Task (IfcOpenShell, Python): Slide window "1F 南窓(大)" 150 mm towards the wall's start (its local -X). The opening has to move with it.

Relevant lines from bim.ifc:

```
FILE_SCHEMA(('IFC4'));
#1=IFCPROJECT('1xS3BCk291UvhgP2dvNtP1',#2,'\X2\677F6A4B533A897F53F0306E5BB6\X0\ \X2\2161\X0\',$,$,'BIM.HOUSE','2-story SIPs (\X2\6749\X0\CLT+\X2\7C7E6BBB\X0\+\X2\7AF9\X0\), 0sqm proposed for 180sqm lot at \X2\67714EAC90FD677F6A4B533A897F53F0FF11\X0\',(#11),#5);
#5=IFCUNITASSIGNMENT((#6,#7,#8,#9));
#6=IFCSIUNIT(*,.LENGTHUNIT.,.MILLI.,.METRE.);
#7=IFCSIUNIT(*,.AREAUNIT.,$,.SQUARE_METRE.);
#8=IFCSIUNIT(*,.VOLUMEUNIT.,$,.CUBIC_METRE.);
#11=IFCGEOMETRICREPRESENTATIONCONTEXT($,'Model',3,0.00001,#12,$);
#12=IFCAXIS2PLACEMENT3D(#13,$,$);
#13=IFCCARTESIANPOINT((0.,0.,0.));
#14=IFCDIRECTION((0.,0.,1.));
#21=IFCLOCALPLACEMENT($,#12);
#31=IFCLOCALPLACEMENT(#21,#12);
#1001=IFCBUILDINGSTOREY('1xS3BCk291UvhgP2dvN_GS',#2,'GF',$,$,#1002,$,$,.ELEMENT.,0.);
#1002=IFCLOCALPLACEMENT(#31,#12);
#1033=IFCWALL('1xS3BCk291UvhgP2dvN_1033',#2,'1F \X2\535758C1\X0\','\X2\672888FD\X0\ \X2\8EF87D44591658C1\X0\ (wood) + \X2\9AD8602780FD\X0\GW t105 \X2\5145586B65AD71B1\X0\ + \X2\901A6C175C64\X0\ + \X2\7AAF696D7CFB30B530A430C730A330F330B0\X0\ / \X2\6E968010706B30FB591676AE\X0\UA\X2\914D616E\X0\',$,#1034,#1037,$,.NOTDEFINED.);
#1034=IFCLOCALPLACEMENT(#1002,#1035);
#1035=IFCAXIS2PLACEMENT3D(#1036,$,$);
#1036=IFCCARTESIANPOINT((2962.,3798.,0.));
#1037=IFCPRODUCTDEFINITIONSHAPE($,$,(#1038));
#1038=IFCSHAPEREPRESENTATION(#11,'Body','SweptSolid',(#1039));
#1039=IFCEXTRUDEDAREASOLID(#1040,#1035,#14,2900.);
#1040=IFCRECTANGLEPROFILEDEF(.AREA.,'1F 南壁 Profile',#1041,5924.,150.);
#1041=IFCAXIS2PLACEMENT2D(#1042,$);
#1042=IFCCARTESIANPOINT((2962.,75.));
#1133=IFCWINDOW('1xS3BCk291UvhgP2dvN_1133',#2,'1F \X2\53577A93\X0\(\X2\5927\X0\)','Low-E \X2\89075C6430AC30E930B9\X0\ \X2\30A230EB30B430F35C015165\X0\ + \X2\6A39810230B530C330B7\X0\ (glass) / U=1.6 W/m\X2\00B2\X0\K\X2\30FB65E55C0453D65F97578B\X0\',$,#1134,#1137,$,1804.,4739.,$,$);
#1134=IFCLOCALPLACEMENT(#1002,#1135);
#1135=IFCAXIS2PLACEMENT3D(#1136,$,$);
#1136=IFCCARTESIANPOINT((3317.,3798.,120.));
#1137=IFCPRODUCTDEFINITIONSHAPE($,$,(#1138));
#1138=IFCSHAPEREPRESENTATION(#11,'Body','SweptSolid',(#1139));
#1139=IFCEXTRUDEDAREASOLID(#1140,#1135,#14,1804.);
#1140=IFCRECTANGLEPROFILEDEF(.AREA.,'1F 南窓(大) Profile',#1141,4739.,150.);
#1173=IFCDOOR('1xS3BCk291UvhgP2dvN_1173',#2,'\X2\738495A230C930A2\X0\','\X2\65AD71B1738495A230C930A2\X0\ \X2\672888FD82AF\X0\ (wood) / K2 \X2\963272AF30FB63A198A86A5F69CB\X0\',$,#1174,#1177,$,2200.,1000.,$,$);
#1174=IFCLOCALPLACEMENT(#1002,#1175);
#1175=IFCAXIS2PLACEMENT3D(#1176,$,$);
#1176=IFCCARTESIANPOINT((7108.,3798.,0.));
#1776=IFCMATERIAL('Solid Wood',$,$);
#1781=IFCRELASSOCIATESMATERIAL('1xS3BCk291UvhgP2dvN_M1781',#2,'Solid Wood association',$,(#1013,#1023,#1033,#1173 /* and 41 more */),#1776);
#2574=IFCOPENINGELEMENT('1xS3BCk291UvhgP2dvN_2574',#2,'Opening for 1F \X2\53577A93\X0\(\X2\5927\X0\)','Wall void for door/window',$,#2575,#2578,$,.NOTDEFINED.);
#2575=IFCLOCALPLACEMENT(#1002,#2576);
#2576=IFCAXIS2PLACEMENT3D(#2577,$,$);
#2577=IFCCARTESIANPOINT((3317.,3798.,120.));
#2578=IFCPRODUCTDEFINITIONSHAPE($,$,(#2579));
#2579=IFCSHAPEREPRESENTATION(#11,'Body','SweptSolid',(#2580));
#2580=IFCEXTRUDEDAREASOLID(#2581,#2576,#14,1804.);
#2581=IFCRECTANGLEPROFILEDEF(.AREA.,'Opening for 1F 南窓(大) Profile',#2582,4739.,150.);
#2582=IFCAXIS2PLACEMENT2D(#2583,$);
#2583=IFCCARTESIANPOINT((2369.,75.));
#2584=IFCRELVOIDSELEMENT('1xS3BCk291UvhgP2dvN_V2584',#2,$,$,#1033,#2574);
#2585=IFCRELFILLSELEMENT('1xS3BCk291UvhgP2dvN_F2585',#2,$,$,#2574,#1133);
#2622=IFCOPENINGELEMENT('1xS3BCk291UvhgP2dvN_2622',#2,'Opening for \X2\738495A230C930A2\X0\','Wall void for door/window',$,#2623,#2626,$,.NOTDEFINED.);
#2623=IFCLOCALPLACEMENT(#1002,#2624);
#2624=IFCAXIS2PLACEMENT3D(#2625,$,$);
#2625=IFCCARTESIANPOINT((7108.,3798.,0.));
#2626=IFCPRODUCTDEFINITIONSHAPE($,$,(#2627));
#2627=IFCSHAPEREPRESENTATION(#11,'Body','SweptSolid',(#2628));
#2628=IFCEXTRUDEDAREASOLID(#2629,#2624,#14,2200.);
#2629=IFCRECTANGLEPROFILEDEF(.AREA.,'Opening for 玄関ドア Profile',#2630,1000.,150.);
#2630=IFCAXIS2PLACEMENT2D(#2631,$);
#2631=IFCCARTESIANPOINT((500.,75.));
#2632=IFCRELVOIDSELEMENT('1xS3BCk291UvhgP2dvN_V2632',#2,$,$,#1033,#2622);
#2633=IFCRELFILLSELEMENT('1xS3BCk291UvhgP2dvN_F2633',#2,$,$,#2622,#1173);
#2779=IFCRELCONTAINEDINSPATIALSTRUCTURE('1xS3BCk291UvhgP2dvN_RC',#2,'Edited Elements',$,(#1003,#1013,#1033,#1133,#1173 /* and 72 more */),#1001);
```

```python
import ifcopenshell
import ifcopenshell.api.geometry
import ifcopenshell.util.placement
import ifcopenshell.util.unit

model = ifcopenshell.open("bim.ifc")
unit_scale = ifcopenshell.util.unit.calculate_unit_scale(model)

window = model.by_guid("1xS3BCk291UvhgP2dvN_1133")
opening = window.FillsVoids[0].RelatingOpeningElement
wall = opening.VoidsElements[0].RelatingBuildingElement

wall_matrix = ifcopenshell.util.placement.get_local_placement(wall.ObjectPlacement)
shift = wall_matrix[:3, 0] * -0.15 / unit_scale
before = ifcopenshell.util.placement.get_local_placement(window.ObjectPlacement)[:3, 3].copy()

# The window is not placed relative to its opening, so move both.
for product in (opening, window):
    matrix = ifcopenshell.util.placement.get_local_placement(product.ObjectPlacement)
    matrix[:3, 3] += shift
    ifcopenshell.api.geometry.edit_object_placement(model, product=product, matrix=matrix, is_si=False)

after = ifcopenshell.util.placement.get_local_placement(window.ObjectPlacement)[:3, 3]
print("window moved by", (after - before).round(3) + 0.0)

model.write("bim-out.ifc")
```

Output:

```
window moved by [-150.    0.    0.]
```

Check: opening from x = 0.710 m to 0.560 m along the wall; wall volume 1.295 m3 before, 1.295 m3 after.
